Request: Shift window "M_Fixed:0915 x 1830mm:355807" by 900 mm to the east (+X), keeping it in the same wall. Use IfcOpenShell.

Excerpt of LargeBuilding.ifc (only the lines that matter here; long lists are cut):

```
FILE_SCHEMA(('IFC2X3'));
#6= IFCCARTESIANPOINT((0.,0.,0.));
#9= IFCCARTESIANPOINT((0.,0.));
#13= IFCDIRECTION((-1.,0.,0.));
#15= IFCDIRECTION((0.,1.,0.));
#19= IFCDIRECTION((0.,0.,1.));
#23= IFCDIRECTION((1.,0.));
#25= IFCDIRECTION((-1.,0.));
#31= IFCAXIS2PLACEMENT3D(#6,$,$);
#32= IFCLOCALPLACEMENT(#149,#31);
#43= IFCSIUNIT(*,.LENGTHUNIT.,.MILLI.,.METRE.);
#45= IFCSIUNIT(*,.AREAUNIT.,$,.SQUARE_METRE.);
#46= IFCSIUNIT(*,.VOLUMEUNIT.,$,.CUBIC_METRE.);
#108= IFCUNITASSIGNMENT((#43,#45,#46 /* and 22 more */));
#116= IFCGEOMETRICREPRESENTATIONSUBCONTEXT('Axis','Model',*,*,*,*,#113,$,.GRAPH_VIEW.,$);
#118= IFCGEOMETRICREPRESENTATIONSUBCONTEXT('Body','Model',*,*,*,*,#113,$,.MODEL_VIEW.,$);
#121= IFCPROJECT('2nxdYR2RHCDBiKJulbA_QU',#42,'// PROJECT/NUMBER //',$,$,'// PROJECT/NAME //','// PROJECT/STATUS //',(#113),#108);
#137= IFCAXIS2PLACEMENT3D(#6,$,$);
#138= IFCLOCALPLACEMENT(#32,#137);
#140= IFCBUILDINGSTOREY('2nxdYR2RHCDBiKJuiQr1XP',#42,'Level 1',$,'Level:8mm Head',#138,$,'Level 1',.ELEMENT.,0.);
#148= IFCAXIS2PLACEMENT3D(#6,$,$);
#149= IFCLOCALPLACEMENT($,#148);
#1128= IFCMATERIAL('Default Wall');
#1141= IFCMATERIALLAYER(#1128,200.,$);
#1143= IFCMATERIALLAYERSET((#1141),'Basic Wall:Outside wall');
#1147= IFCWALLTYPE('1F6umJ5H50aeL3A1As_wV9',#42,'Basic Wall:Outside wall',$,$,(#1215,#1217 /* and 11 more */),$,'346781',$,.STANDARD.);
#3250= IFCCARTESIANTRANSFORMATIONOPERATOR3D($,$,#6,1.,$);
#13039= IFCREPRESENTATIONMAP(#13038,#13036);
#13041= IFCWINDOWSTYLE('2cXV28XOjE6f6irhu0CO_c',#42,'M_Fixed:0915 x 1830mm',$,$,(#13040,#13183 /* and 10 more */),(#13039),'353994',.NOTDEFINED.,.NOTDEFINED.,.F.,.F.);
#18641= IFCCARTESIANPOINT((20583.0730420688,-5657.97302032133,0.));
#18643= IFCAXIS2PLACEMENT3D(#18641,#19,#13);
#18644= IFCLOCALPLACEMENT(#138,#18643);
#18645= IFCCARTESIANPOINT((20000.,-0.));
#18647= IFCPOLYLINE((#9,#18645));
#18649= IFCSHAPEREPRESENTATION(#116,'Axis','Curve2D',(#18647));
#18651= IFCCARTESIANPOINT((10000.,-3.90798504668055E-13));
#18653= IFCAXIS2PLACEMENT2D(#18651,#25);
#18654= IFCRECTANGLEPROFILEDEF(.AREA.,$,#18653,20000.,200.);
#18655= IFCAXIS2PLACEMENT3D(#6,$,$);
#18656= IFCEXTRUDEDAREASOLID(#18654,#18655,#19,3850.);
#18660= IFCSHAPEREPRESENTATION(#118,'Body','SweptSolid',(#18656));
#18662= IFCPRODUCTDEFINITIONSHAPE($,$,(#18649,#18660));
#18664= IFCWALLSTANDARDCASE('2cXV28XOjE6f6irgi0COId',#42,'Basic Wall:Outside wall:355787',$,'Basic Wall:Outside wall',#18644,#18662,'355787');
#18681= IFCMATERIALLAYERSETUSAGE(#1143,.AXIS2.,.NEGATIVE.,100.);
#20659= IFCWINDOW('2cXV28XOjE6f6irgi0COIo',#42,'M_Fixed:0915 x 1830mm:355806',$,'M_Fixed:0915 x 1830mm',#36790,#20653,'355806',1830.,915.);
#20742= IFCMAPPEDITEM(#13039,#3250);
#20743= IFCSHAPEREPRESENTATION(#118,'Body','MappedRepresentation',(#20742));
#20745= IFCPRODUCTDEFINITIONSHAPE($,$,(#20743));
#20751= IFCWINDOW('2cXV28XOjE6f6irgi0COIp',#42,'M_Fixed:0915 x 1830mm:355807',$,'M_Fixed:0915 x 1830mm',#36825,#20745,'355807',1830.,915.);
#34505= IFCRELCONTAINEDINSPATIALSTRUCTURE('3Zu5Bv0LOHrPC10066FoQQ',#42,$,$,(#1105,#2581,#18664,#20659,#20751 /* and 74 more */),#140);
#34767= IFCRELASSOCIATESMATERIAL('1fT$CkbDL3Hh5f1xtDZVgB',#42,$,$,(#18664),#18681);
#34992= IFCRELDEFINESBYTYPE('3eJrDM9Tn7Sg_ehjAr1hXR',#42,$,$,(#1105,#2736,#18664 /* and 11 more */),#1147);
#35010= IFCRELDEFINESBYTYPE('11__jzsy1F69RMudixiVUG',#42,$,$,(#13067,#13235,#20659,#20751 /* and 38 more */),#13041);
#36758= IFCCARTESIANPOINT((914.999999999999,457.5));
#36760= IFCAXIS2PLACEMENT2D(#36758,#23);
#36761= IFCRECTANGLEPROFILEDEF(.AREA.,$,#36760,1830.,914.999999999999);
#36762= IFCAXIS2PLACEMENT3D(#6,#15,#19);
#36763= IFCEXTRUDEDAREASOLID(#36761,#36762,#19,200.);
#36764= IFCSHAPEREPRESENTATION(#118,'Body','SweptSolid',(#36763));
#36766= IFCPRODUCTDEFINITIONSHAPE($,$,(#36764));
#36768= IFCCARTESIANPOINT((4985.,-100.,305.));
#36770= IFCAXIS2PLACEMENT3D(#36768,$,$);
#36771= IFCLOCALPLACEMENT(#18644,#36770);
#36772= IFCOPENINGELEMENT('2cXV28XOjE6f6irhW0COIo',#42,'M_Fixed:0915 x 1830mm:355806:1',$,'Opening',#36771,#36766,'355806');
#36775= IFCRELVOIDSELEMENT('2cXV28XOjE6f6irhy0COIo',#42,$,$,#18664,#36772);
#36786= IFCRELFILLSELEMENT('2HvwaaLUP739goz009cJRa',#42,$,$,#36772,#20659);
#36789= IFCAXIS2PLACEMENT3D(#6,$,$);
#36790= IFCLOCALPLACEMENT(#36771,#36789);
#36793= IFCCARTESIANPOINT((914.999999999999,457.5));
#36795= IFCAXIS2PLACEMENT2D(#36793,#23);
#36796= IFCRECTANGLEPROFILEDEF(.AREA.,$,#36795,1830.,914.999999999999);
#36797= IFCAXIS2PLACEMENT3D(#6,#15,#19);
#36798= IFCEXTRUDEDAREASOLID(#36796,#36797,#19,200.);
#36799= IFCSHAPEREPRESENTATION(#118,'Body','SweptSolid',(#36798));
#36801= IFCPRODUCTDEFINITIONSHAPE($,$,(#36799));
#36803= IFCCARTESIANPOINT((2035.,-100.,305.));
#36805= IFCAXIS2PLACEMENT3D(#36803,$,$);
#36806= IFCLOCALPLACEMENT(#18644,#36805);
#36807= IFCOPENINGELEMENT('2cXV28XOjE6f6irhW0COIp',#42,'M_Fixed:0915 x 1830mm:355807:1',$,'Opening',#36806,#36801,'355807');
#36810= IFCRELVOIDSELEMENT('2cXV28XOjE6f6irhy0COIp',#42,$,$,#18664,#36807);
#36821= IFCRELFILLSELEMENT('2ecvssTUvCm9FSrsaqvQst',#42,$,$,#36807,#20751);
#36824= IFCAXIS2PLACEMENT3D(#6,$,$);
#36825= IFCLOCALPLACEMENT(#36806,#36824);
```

```python
import ifcopenshell
import ifcopenshell.api.geometry
import ifcopenshell.util.placement
import ifcopenshell.util.unit

model = ifcopenshell.open("LargeBuilding.ifc")
unit_scale = ifcopenshell.util.unit.calculate_unit_scale(model)

window = model.by_guid("2cXV28XOjE6f6irgi0COIp")
opening = window.FillsVoids[0].RelatingOpeningElement
wall = opening.VoidsElements[0].RelatingBuildingElement

wall_matrix = ifcopenshell.util.placement.get_local_placement(wall.ObjectPlacement)
shift = wall_matrix[:3, 0] * -0.9 / unit_scale
before = ifcopenshell.util.placement.get_local_placement(window.ObjectPlacement)[:3, 3].copy()

# The window is placed relative to its opening, so it follows when the opening moves.
matrix = ifcopenshell.util.placement.get_local_placement(opening.ObjectPlacement)
matrix[:3, 3] += shift
ifcopenshell.api.geometry.edit_object_placement(
    model, product=opening, matrix=matrix, is_si=False, should_transform_children=True
)

after = ifcopenshell.util.placement.get_local_placement(window.ObjectPlacement)[:3, 3]
print("window moved by", (after - before).round(3) + 0.0)

model.write("LargeBuilding_v2.ifc")
```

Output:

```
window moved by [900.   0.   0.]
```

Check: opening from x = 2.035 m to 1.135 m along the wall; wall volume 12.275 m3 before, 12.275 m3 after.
